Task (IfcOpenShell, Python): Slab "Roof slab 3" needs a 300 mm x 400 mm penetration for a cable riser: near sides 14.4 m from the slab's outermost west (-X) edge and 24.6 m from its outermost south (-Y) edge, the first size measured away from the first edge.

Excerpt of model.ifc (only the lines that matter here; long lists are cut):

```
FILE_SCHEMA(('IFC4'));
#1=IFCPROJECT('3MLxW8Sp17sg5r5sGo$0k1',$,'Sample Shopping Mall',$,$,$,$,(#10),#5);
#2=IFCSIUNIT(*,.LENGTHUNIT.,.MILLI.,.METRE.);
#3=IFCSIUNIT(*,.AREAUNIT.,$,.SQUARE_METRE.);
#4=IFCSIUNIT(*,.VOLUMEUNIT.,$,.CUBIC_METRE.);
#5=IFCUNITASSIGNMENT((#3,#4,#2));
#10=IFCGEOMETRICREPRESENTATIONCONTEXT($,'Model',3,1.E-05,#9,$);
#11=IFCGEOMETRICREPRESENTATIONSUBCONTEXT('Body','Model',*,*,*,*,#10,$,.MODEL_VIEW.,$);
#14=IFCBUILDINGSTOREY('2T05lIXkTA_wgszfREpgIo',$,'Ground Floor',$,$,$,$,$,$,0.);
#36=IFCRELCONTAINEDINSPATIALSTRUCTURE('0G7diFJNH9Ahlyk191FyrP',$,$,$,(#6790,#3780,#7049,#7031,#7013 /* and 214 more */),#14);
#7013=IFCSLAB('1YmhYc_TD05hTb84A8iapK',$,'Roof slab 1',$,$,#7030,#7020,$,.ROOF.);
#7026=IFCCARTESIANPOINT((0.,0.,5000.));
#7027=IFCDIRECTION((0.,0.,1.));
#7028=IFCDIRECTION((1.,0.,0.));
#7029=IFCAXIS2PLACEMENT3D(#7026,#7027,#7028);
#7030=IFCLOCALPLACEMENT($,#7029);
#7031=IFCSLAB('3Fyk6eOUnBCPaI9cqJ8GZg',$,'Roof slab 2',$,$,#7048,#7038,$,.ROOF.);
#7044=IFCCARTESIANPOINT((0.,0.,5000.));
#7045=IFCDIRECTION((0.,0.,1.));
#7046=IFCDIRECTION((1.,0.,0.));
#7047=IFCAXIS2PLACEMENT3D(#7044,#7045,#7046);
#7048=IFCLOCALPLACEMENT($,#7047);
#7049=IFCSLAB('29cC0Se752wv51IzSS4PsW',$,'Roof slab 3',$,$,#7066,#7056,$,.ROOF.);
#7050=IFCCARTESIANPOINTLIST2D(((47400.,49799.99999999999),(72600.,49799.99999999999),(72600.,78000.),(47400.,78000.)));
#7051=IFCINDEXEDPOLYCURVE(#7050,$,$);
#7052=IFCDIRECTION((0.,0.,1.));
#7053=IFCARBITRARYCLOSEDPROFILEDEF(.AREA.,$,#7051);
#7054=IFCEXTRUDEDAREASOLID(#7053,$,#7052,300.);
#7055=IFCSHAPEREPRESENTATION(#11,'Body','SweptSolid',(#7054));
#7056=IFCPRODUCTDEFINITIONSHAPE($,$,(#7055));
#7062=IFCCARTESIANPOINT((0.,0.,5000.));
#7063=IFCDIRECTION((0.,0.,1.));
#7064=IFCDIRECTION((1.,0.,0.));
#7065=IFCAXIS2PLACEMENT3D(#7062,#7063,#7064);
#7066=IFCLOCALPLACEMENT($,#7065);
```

```python
import numpy as np
import ifcopenshell
import ifcopenshell.api.feature
import ifcopenshell.api.geometry
import ifcopenshell.api.root
import ifcopenshell.geom
import ifcopenshell.util.placement
import ifcopenshell.util.representation
import ifcopenshell.util.shape
import ifcopenshell.util.unit

model = ifcopenshell.open("model.ifc")
unit_scale = ifcopenshell.util.unit.calculate_unit_scale(model)
settings = ifcopenshell.geom.settings()


def volume(element):
    """Net volume in cubic metres, openings subtracted."""
    shape = ifcopenshell.geom.create_shape(settings, element)
    return ifcopenshell.util.shape.get_volume(shape.geometry)


slab = model.by_guid("29cC0Se752wv51IzSS4PsW")
before = volume(slab)

# Extent in the slab's own axes, in metres. The edges named are its -X and -Y sides.
slab_shape = ifcopenshell.geom.create_shape(settings, slab)
vertices = ifcopenshell.util.shape.get_vertices(slab_shape.geometry)
x_min, y_min, bottom = vertices.min(axis=0)
top = vertices[:, 2].max()

opening = ifcopenshell.api.root.create_entity(model, ifc_class="IfcOpeningElement", name="Cable riser opening", predefined_type="OPENING")
context = ifcopenshell.util.representation.get_context(model, "Model", "Body", "MODEL_VIEW")
width, depth = 0.3, 0.4
outline = [(0.0, 0.0), (width, 0.0), (width, depth), (0.0, depth), (0.0, 0.0)]
# Overshoot both faces by 50 mm so the cut is clean.
shape = ifcopenshell.api.geometry.add_slab_representation(
    model, context=context, depth=top - bottom + 0.1, polyline=outline
)
ifcopenshell.api.geometry.assign_representation(model, product=opening, representation=shape)

matrix = ifcopenshell.util.placement.get_local_placement(slab.ObjectPlacement)
matrix[:, 3] = matrix @ np.append(np.array([x_min + 14.4, y_min + 24.6, bottom - 0.05]) / unit_scale, 1.0)
ifcopenshell.api.geometry.edit_object_placement(model, product=opening, matrix=matrix, is_si=False)
ifcopenshell.api.feature.add_feature(model, feature=opening, element=slab)

after = volume(slab)

print(f"slab volume {before:.3f} -> {after:.3f} m3")

model.write("model_edited.ifc")
```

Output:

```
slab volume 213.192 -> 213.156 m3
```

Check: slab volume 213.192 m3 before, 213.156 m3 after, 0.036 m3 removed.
